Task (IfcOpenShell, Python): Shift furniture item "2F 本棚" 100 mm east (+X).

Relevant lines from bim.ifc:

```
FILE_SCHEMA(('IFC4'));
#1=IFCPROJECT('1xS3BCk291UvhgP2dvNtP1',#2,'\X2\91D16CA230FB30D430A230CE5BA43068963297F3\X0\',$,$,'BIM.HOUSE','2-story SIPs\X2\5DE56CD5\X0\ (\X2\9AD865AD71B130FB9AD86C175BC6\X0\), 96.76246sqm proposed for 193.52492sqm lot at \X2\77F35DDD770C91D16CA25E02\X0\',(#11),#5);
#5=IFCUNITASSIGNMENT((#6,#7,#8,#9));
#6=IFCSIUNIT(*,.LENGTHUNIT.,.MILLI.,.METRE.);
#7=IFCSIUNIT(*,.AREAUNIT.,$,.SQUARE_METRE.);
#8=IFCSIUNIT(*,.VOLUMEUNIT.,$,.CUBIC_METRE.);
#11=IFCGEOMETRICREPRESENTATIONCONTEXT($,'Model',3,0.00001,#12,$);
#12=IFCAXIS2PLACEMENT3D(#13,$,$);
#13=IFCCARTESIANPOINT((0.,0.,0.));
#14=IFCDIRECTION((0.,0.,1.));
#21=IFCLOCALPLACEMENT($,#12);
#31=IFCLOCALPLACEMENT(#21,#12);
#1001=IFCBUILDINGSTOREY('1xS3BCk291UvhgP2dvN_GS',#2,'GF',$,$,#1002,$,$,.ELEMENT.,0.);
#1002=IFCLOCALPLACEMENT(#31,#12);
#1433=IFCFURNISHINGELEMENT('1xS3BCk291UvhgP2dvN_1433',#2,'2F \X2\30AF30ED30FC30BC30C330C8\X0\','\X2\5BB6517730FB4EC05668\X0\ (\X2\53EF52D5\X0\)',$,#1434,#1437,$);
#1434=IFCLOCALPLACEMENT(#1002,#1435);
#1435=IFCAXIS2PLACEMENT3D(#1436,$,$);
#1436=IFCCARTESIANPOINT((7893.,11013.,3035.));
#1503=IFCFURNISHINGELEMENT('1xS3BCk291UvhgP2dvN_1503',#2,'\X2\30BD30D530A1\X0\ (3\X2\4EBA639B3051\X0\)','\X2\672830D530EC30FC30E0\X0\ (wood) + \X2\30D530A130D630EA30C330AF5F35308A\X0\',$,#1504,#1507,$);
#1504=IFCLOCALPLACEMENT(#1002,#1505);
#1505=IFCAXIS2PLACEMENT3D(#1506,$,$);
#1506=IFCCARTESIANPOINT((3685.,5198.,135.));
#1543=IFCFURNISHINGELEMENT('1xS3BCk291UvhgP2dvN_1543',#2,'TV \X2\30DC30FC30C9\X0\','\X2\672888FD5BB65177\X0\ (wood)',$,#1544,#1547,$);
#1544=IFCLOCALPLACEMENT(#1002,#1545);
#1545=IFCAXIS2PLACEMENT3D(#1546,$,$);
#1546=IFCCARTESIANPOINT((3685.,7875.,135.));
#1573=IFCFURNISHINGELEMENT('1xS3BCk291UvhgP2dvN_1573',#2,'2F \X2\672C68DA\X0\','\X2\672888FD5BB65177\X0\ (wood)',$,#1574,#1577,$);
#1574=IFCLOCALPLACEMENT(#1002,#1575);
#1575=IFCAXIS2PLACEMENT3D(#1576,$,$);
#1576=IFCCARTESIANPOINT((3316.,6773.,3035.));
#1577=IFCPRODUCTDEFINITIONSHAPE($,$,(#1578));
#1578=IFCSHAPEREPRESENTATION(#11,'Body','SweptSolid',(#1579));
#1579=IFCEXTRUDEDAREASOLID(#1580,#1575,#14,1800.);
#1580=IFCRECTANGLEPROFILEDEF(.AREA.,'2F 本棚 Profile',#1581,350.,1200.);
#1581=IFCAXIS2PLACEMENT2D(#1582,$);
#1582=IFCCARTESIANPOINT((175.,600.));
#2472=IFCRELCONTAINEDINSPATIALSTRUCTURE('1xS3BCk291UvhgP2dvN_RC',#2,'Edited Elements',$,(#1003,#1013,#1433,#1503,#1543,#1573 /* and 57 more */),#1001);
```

```python
import ifcopenshell
import ifcopenshell.api.geometry
import ifcopenshell.util.placement
import ifcopenshell.util.unit

model = ifcopenshell.open("bim.ifc")
unit_scale = ifcopenshell.util.unit.calculate_unit_scale(model)

item = model.by_guid("1xS3BCk291UvhgP2dvN_1573")
matrix = ifcopenshell.util.placement.get_local_placement(item.ObjectPlacement)
matrix[0, 3] += 0.1 / unit_scale
ifcopenshell.api.geometry.edit_object_placement(model, product=item, matrix=matrix, is_si=False)

print(ifcopenshell.util.placement.get_local_placement(item.ObjectPlacement).round(3) + 0.0)

model.write("bim_edited.ifc")
```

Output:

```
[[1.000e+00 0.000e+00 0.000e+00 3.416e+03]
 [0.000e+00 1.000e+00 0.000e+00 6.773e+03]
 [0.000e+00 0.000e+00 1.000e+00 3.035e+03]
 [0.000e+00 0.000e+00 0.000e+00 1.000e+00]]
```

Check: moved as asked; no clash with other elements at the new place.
